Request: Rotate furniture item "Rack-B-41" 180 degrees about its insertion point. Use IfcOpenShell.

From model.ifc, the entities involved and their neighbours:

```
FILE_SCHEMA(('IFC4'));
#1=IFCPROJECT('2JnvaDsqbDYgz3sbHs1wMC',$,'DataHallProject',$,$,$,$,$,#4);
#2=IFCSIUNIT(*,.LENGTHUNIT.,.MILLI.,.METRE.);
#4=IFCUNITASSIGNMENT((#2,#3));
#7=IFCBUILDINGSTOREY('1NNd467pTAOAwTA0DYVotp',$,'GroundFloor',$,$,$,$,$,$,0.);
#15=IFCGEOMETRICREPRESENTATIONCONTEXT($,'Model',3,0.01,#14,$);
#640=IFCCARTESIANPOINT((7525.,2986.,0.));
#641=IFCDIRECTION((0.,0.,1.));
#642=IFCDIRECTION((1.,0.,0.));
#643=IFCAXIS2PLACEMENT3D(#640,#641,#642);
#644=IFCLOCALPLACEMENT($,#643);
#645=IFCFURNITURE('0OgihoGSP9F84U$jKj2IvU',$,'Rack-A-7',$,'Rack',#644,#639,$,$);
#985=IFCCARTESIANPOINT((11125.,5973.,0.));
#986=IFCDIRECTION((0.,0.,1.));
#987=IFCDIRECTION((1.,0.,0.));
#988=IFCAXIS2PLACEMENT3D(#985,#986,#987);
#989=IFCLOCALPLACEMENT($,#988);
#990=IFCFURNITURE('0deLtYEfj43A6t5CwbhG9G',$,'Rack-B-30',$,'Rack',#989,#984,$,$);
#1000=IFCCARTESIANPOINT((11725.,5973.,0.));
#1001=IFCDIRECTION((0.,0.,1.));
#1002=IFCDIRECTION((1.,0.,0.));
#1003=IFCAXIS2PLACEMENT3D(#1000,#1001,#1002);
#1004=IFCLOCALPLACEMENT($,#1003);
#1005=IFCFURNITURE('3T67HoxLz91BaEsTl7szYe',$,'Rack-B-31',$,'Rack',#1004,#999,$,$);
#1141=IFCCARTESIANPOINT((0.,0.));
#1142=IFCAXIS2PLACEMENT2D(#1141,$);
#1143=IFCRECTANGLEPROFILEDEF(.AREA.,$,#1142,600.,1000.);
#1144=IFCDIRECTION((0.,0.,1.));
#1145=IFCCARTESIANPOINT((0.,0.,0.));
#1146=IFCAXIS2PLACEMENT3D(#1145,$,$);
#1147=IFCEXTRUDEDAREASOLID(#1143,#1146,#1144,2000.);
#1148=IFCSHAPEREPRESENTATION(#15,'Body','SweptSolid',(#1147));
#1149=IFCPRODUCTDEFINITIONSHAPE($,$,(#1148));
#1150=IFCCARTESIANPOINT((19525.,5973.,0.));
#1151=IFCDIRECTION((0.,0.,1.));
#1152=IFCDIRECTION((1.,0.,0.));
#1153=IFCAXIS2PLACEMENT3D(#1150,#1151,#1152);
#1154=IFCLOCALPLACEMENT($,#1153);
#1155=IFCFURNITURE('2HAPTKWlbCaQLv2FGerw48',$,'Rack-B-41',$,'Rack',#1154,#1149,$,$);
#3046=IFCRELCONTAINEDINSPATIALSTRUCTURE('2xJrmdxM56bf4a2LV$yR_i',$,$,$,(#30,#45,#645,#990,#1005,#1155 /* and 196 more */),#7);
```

```python
import ifcopenshell
import ifcopenshell.api.geometry
import ifcopenshell.util.placement

model = ifcopenshell.open("model.ifc")

item = model.by_guid("2HAPTKWlbCaQLv2FGerw48")
matrix = ifcopenshell.util.placement.get_local_placement(item.ObjectPlacement)
matrix = matrix @ ifcopenshell.util.placement.rotation(180, "Z")
ifcopenshell.api.geometry.edit_object_placement(model, product=item, matrix=matrix, is_si=False)

print(ifcopenshell.util.placement.get_local_placement(item.ObjectPlacement).round(3) + 0.0)

model.write("model_updated.ifc")
```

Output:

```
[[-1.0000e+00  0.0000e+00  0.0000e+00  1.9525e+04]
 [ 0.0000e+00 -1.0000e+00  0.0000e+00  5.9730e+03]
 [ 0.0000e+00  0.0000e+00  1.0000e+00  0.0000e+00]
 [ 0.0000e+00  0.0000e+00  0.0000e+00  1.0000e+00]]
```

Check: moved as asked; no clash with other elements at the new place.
